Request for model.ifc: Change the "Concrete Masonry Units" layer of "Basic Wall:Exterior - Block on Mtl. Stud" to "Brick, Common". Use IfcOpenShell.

First a look at what the model holds.

```python
import ifcopenshell
import ifcopenshell.util.element

model = ifcopenshell.open("model.ifc")
print(model.schema)
for layer_set in model.by_type("IfcMaterialLayerSet"):
    if layer_set.LayerSetName == "Basic Wall:Exterior - Block on Mtl. Stud":
        for layer in layer_set.MaterialLayers:
            print(layer.id(), layer.Material and layer.Material.Name, layer.LayerThickness, sep=" | ")
        print(len(ifcopenshell.util.element.get_elements_by_material(model, layer_set)), "elements and types use it")
print(sorted(m.Name for m in model.by_type("IfcMaterial") if m.Name)[:60])
```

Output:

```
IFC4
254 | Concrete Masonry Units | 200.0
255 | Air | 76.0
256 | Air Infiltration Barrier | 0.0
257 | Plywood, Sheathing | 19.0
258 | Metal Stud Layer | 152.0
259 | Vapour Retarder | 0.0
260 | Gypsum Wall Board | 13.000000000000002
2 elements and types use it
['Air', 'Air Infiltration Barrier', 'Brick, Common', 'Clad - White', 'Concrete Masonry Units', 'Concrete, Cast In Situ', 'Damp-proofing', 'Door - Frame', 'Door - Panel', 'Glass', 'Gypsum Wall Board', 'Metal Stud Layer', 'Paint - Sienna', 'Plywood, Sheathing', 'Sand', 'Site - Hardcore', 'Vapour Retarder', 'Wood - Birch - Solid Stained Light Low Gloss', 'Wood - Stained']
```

```python
import ifcopenshell
import ifcopenshell.api.material

model = ifcopenshell.open("model.ifc")

layer_set = next(s for s in model.by_type("IfcMaterialLayerSet") if s.LayerSetName == "Basic Wall:Exterior - Block on Mtl. Stud")
layer = next(l for l in layer_set.MaterialLayers if l.Material and l.Material.Name == "Concrete Masonry Units")
material = next(m for m in model.by_type("IfcMaterial") if m.Name == "Brick, Common")

# Point this one layer at the other material; renaming the old one would change it everywhere.
ifcopenshell.api.material.edit_layer(model, layer=layer, attributes={"Name": material.Name}, material=material)

print([l.Material.Name if l.Material else None for l in layer_set.MaterialLayers])

model.write("model_v2.ifc")
```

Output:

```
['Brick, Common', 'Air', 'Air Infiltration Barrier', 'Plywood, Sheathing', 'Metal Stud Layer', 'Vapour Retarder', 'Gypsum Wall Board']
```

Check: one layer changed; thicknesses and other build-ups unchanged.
